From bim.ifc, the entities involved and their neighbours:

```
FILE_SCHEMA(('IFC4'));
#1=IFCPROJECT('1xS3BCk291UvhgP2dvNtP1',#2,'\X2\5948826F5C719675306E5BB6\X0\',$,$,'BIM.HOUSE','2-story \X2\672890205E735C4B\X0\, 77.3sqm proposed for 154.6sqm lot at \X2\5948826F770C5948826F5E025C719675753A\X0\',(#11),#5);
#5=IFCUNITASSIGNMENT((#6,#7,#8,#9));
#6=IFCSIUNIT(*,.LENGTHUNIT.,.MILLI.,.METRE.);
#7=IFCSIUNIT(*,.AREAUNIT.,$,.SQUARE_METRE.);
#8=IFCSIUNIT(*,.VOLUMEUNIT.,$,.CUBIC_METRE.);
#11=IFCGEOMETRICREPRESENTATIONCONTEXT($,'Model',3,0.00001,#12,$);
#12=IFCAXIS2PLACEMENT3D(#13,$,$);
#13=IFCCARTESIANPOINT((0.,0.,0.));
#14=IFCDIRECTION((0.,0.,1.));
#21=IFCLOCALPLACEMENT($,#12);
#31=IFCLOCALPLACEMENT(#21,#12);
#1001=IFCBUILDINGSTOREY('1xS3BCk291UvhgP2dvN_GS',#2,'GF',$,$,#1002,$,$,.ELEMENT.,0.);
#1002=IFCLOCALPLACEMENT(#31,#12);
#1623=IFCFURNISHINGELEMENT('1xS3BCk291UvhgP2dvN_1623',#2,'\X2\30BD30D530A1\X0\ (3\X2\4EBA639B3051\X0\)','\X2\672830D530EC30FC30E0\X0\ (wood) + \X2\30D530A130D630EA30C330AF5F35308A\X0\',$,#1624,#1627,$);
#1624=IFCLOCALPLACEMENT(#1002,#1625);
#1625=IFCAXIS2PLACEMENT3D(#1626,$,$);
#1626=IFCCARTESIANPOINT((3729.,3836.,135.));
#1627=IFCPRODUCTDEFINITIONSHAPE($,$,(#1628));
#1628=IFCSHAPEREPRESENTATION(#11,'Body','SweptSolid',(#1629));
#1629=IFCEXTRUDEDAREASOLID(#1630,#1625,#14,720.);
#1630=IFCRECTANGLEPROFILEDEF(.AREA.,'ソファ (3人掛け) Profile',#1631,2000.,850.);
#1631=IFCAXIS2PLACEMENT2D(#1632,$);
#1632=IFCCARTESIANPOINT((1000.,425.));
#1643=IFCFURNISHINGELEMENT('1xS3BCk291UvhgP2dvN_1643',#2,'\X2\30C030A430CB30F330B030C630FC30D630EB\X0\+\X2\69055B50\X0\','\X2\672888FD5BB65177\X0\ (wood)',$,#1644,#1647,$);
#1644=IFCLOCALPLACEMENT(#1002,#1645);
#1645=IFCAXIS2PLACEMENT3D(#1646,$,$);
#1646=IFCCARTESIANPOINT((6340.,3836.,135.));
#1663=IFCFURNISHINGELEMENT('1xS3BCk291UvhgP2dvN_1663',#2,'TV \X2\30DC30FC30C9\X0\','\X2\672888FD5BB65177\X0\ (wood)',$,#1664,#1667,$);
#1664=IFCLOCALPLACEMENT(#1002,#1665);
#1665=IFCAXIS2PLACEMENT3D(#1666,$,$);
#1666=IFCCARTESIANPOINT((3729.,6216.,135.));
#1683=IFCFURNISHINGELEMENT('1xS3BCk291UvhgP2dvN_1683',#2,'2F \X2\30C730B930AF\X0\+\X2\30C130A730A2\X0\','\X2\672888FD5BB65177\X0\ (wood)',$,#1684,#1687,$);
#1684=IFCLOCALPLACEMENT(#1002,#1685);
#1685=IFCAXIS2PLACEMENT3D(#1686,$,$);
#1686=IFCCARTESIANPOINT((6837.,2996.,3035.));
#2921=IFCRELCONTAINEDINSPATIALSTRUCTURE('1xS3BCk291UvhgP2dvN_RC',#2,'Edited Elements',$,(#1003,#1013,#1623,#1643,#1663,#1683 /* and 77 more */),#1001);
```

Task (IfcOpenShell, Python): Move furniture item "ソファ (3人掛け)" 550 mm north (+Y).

```python
import ifcopenshell
import ifcopenshell.api.geometry
import ifcopenshell.util.placement

model = ifcopenshell.open("bim.ifc")

item = model.by_guid("1xS3BCk291UvhgP2dvN_1623")
matrix = ifcopenshell.util.placement.get_local_placement(item.ObjectPlacement)
matrix[1, 3] += 550.0
ifcopenshell.api.geometry.edit_object_placement(model, product=item, matrix=matrix, is_si=False)

print(ifcopenshell.util.placement.get_local_placement(item.ObjectPlacement).round(3) + 0.0)

model.write("bim-out.ifc")
```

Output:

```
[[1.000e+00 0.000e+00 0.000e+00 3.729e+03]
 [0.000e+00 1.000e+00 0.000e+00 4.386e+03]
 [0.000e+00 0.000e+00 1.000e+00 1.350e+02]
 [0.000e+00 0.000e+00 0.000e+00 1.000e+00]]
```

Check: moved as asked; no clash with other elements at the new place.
